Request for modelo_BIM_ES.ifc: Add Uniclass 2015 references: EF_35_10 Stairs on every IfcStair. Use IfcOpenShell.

First a look at what the model holds.

```python
import ifcopenshell

model = ifcopenshell.open("modelo_BIM_ES.ifc")
print(model.schema)
print("classifications:", [c.Name for c in model.by_type("IfcClassification")])
for ifc_class in ("IfcDoor", "IfcRoof", "IfcStair", "IfcWall", "IfcWindow"):
    print(ifc_class, len(model.by_type(ifc_class)))
```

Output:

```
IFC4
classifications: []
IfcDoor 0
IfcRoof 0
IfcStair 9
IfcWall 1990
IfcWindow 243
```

```python
import ifcopenshell
import ifcopenshell.api.classification

model = ifcopenshell.open("modelo_BIM_ES.ifc")

system = ifcopenshell.api.classification.add_classification(model, classification="Uniclass 2015")

codes = {
    "IfcStair": ("EF_35_10", "Stairs"),
}
for ifc_class, (code, name) in codes.items():
    products = model.by_type(ifc_class)
    ifcopenshell.api.classification.add_reference(
        model, products=products, classification=system, identification=code, name=name
    )
    print(code, len(products))

model.write("modelo_BIM_ES_updated.ifc")
```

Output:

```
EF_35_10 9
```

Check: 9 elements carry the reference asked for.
